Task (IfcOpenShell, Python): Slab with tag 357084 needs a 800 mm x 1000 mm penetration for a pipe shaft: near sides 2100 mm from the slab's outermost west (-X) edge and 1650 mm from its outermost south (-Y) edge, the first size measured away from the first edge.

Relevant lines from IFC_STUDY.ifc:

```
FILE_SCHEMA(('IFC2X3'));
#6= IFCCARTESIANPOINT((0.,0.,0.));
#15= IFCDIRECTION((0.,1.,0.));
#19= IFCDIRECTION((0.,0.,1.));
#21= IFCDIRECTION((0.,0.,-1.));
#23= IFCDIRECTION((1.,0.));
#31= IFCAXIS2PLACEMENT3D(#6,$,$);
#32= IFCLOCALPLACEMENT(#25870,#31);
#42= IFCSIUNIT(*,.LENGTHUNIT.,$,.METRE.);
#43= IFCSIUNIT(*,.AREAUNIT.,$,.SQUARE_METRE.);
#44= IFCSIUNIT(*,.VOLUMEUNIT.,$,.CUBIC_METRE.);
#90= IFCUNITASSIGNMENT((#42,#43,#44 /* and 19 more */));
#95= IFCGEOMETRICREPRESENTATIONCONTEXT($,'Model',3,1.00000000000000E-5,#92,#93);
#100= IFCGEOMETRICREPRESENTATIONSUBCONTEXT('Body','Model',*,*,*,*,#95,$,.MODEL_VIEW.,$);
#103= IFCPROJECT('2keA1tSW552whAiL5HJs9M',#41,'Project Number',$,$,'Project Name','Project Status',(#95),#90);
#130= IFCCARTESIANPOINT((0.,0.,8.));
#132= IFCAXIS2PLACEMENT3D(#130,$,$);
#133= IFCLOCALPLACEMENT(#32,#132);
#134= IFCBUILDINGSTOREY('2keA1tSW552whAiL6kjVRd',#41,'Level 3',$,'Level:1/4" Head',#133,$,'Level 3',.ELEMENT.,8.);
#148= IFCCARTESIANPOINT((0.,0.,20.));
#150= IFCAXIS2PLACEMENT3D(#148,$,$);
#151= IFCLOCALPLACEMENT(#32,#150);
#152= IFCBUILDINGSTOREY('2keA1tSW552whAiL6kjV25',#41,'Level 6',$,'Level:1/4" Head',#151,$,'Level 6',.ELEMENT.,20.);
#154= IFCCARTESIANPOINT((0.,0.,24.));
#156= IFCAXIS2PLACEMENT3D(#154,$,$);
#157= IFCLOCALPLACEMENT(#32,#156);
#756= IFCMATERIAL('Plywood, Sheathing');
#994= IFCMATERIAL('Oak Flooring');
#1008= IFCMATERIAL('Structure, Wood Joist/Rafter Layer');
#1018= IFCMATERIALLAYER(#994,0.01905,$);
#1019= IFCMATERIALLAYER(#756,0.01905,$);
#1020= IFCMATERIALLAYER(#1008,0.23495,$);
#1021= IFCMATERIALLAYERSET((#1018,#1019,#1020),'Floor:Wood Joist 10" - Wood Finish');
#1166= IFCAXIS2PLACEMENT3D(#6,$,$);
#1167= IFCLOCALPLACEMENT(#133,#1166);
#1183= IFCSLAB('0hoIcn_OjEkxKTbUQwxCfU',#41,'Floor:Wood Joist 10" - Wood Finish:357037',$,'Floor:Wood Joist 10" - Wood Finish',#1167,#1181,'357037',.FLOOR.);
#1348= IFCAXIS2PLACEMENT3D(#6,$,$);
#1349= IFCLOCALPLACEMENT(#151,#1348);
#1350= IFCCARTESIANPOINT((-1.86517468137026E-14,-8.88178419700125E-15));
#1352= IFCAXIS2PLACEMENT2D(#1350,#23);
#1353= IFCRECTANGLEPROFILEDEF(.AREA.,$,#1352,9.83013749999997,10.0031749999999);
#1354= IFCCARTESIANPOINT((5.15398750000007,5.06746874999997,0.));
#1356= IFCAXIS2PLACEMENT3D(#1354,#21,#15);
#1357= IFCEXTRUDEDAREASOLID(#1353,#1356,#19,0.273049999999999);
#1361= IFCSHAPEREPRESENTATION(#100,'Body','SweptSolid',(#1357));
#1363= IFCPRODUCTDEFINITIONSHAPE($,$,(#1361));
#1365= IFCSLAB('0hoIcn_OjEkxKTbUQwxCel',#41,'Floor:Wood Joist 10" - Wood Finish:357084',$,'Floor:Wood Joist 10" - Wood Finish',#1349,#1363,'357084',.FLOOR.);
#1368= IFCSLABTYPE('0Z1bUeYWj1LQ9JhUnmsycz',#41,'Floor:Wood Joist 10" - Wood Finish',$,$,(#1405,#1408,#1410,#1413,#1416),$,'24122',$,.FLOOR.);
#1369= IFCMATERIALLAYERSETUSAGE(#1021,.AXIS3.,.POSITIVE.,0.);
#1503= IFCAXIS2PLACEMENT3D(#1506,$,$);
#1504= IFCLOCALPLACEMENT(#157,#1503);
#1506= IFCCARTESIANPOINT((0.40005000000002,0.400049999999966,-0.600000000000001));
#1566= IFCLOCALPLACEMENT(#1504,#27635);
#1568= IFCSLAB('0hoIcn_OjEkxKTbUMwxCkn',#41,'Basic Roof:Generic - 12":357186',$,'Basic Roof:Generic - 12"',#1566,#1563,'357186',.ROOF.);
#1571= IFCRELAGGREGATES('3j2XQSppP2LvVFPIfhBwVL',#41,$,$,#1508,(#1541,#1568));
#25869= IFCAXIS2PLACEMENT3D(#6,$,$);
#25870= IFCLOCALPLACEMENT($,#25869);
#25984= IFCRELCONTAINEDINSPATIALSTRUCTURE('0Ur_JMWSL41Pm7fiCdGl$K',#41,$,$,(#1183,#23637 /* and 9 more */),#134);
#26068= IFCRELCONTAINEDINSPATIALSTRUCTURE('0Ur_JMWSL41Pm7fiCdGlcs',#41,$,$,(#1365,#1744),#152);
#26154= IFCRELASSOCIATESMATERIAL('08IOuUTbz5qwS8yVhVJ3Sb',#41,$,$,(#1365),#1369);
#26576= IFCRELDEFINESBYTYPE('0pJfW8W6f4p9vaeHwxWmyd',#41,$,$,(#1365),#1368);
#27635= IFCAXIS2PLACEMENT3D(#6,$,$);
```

```python
import numpy as np
import ifcopenshell
import ifcopenshell.api.feature
import ifcopenshell.api.geometry
import ifcopenshell.api.root
import ifcopenshell.geom
import ifcopenshell.util.placement
import ifcopenshell.util.representation
import ifcopenshell.util.shape
import ifcopenshell.util.unit

model = ifcopenshell.open("IFC_STUDY.ifc")
unit_scale = ifcopenshell.util.unit.calculate_unit_scale(model)
settings = ifcopenshell.geom.settings()


def volume(element):
    """Net volume in cubic metres, openings subtracted."""
    shape = ifcopenshell.geom.create_shape(settings, element)
    return ifcopenshell.util.shape.get_volume(shape.geometry)


slab = model.by_guid("0hoIcn_OjEkxKTbUQwxCel")
before = volume(slab)

# Extent in the slab's own axes, in metres. The edges named are its -X and -Y sides.
slab_shape = ifcopenshell.geom.create_shape(settings, slab)
vertices = ifcopenshell.util.shape.get_vertices(slab_shape.geometry)
x_min, y_min, bottom = vertices.min(axis=0)
top = vertices[:, 2].max()

opening = ifcopenshell.api.root.create_entity(model, ifc_class="IfcOpeningElement", name="Pipe shaft opening")
context = ifcopenshell.util.representation.get_context(model, "Model", "Body", "MODEL_VIEW")
width, depth = 0.8, 1
outline = [(0.0, 0.0), (width, 0.0), (width, depth), (0.0, depth), (0.0, 0.0)]
# Overshoot both faces by 50 mm so the cut is clean.
shape = ifcopenshell.api.geometry.add_slab_representation(
    model, context=context, depth=top - bottom + 0.1, polyline=outline
)
ifcopenshell.api.geometry.assign_representation(model, product=opening, representation=shape)

matrix = ifcopenshell.util.placement.get_local_placement(slab.ObjectPlacement)
matrix[:, 3] = matrix @ np.append(np.array([x_min + 2.1, y_min + 1.65, bottom - 0.05]) / unit_scale, 1.0)
ifcopenshell.api.geometry.edit_object_placement(model, product=opening, matrix=matrix, is_si=False)
ifcopenshell.api.feature.add_feature(model, feature=opening, element=slab)

after = volume(slab)

print(f"slab volume {before:.3f} -> {after:.3f} m3")

model.write("IFC_STUDY_edited.ifc")
```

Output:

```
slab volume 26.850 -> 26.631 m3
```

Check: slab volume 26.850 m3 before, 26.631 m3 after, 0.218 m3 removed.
